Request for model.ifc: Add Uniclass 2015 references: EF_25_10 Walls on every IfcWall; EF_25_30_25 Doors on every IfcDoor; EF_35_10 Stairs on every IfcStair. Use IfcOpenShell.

First a look at what the model holds.

```python
import ifcopenshell

model = ifcopenshell.open("model.ifc")
print(model.schema)
print("classifications:", [c.Name for c in model.by_type("IfcClassification")])
for ifc_class in ("IfcDoor", "IfcRoof", "IfcStair", "IfcWall", "IfcWindow"):
    print(ifc_class, len(model.by_type(ifc_class)))
```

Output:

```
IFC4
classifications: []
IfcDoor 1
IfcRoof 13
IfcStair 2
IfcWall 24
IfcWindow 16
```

```python
import ifcopenshell
import ifcopenshell.api.classification

model = ifcopenshell.open("model.ifc")

system = ifcopenshell.api.classification.add_classification(model, classification="Uniclass 2015")

codes = {
    "IfcWall": ("EF_25_10", "Walls"),
    "IfcDoor": ("EF_25_30_25", "Doors"),
    "IfcStair": ("EF_35_10", "Stairs"),
}
for ifc_class, (code, name) in codes.items():
    products = model.by_type(ifc_class)
    ifcopenshell.api.classification.add_reference(
        model, products=products, classification=system, identification=code, name=name
    )
    print(code, len(products))

model.write("model_edited.ifc")
```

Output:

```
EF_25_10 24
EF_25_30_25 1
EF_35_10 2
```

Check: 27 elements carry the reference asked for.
